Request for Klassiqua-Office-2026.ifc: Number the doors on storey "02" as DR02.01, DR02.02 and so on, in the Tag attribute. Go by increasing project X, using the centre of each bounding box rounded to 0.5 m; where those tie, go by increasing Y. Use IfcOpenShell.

First a look at what the model holds.

```python
import ifcopenshell
import ifcopenshell.util.element
import ifcopenshell.util.placement

model = ifcopenshell.open("Klassiqua-Office-2026.ifc")
print(model.schema)
storey = next(s for s in model.by_type("IfcBuildingStorey") if s.Name == "02")
doors = [e for e in ifcopenshell.util.element.get_decomposition(storey) if e.is_a("IfcDoor")]
for e in sorted(doors, key=lambda e: e.id()):
    origin = ifcopenshell.util.placement.get_local_placement(e.ObjectPlacement)[:3, 3]
    print(e.id(), e.Tag, e.Name, origin.round(2) + 0.0, sep=" | ")
```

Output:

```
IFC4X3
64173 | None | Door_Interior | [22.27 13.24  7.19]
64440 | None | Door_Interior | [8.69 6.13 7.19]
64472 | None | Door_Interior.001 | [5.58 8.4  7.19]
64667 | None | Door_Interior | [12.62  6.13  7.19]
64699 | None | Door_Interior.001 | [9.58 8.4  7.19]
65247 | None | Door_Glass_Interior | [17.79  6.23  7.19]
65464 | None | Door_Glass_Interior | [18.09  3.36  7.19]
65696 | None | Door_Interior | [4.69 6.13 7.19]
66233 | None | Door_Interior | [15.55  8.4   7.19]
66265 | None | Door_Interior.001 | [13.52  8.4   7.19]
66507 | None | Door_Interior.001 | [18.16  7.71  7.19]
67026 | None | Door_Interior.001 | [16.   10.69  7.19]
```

```python
import ifcopenshell
import ifcopenshell.geom
import ifcopenshell.util.element
import ifcopenshell.util.shape

model = ifcopenshell.open("Klassiqua-Office-2026.ifc")
settings = ifcopenshell.geom.settings()
settings.set("use-world-coords", True)


def centre(element):
    shape = ifcopenshell.geom.create_shape(settings, element)
    return ifcopenshell.util.shape.get_bbox_centroid(shape.geometry)


storey = next(s for s in model.by_type("IfcBuildingStorey") if s.Name == "02")
doors = [e for e in ifcopenshell.util.element.get_decomposition(storey) if e.is_a("IfcDoor")]

# Insertion points can sit at a corner or the storey origin, so sort by the geometry (in metres).
centres = {e: centre(e) for e in doors}
doors.sort(key=lambda e: (round(centres[e][0] / 0.5), centres[e][1]))

for i, e in enumerate(doors, start=1):
    number = f"DR02.{i:02d}"
    e.Tag = number
    print(e.id(), number)

model.write("Klassiqua-Office-2026_updated.ifc")
```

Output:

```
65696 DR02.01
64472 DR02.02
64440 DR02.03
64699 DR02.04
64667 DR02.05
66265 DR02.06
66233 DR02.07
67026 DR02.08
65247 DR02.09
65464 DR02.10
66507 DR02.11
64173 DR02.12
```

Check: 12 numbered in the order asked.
